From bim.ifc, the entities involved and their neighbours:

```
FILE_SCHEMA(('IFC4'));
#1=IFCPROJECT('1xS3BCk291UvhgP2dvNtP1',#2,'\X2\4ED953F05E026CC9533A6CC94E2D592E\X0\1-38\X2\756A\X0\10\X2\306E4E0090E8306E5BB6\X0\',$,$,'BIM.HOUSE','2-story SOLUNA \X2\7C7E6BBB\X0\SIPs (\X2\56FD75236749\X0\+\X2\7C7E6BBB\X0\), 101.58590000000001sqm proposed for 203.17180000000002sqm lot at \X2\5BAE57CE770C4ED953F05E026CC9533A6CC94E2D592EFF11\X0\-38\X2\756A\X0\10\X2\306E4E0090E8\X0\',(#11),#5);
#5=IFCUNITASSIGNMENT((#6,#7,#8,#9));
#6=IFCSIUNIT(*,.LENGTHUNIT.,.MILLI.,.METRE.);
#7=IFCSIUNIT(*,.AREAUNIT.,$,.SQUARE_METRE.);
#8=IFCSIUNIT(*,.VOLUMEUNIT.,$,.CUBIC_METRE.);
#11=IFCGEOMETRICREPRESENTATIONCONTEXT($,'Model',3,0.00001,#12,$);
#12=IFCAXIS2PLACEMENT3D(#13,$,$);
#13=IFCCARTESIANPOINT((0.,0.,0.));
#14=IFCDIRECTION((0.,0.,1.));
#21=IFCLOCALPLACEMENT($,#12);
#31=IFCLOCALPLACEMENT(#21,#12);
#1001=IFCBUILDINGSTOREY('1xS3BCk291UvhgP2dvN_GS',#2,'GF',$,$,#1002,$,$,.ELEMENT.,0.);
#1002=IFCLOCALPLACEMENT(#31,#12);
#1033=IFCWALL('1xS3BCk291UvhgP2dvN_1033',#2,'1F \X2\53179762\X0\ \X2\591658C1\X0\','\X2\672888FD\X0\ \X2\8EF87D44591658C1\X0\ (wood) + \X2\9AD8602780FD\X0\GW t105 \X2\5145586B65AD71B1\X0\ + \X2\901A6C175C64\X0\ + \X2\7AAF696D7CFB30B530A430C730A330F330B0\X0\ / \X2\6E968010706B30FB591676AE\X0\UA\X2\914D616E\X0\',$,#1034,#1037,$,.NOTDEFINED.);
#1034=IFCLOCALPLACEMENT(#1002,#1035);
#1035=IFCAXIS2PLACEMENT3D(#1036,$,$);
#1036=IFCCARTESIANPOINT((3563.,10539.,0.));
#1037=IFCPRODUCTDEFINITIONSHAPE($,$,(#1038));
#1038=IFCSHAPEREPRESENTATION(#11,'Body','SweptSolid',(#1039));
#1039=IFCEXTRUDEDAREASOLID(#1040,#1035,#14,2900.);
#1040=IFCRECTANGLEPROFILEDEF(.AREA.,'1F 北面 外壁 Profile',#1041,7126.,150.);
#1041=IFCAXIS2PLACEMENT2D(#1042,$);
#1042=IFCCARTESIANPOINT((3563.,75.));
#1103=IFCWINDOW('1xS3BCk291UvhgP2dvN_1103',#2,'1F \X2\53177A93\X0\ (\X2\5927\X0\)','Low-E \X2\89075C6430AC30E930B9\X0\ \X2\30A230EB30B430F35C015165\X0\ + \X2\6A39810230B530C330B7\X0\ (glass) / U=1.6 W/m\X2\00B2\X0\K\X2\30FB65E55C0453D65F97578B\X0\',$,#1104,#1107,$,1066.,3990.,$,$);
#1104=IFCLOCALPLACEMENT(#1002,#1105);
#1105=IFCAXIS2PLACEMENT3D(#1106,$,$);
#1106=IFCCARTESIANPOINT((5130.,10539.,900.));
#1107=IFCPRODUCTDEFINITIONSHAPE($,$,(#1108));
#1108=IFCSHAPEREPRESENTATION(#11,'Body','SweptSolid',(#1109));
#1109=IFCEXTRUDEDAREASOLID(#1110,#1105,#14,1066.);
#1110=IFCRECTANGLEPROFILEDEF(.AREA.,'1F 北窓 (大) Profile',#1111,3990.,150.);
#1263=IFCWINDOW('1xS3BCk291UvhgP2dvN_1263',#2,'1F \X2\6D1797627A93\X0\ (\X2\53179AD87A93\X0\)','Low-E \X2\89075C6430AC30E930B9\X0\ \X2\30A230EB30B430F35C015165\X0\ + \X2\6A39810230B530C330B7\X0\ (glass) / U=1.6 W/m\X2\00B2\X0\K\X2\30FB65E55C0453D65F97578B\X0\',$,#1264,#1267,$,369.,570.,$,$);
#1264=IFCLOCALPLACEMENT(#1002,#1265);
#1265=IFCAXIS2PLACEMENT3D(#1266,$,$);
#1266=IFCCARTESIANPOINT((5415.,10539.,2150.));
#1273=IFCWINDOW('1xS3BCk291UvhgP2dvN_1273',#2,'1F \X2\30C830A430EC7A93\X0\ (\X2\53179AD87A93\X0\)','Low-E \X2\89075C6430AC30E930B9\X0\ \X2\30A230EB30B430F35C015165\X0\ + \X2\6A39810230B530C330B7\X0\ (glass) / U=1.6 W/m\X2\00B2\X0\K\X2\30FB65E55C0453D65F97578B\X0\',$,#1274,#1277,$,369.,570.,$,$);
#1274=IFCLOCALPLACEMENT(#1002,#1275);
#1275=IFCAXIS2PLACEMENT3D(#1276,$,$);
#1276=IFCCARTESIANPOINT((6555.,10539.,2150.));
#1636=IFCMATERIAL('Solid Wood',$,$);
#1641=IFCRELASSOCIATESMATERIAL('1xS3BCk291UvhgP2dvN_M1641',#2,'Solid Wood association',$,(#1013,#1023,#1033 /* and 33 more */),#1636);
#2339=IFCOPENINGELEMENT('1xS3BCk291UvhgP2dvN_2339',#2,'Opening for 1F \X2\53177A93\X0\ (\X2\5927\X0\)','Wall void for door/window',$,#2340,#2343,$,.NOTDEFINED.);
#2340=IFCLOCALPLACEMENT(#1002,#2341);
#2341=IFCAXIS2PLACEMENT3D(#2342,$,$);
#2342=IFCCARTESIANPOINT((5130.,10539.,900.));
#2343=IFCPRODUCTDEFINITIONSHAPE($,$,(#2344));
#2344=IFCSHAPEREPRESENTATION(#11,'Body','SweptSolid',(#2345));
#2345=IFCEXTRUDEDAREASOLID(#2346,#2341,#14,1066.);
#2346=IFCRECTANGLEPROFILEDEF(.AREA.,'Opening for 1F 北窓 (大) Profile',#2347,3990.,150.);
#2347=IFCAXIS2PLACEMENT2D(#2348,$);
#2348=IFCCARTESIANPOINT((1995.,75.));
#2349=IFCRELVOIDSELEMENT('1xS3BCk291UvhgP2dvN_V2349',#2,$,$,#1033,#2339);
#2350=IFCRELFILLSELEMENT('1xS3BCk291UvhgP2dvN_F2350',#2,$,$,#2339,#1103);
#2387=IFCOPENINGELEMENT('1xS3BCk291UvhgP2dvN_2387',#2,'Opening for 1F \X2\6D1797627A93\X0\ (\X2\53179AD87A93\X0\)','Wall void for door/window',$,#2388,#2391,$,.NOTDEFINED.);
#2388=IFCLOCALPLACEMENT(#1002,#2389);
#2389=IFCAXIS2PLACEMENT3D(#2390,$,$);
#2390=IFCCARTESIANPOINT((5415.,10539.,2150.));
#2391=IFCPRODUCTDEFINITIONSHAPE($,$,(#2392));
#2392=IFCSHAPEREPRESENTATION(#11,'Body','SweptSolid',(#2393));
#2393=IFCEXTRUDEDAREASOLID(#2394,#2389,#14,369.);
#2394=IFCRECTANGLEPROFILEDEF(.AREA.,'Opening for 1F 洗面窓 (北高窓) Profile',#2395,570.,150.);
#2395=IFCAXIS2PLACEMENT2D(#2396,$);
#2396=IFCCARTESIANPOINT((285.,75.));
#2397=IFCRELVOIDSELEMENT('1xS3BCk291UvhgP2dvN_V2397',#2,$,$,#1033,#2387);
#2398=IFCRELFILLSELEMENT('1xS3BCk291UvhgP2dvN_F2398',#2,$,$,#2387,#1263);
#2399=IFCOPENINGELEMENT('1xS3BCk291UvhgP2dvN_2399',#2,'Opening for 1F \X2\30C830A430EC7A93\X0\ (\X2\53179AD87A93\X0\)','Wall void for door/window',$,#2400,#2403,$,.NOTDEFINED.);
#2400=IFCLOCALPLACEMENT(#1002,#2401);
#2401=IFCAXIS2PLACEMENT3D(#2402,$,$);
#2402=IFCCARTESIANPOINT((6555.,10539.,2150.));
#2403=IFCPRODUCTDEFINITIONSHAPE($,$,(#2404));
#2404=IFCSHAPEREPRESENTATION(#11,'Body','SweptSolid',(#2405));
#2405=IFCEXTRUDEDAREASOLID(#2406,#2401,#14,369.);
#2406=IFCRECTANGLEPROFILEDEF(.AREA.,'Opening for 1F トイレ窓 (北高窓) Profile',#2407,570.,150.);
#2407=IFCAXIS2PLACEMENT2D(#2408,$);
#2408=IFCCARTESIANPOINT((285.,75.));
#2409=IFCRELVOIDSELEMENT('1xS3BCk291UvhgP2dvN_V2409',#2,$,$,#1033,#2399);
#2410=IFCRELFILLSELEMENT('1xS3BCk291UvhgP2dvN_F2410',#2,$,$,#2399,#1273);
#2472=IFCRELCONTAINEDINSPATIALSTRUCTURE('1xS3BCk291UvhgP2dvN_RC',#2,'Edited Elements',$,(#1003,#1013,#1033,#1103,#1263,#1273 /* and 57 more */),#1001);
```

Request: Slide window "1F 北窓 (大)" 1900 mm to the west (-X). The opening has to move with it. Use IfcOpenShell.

```python
import ifcopenshell
import ifcopenshell.api.geometry
import ifcopenshell.util.placement

model = ifcopenshell.open("bim.ifc")

window = model.by_id(1103)
opening = window.FillsVoids[0].RelatingOpeningElement
wall = opening.VoidsElements[0].RelatingBuildingElement

wall_matrix = ifcopenshell.util.placement.get_local_placement(wall.ObjectPlacement)
shift = wall_matrix[:3, 0] * -1900.0
before = ifcopenshell.util.placement.get_local_placement(window.ObjectPlacement)[:3, 3].copy()

# The window is not placed relative to its opening, so move both.
for product in (opening, window):
    matrix = ifcopenshell.util.placement.get_local_placement(product.ObjectPlacement)
    matrix[:3, 3] += shift
    ifcopenshell.api.geometry.edit_object_placement(model, product=product, matrix=matrix, is_si=False)

after = ifcopenshell.util.placement.get_local_placement(window.ObjectPlacement)[:3, 3]
print("window moved by", (after - before).round(3) + 0.0)

model.write("bim-out.ifc")
```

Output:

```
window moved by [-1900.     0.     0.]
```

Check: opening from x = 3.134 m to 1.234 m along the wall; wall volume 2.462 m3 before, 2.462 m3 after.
